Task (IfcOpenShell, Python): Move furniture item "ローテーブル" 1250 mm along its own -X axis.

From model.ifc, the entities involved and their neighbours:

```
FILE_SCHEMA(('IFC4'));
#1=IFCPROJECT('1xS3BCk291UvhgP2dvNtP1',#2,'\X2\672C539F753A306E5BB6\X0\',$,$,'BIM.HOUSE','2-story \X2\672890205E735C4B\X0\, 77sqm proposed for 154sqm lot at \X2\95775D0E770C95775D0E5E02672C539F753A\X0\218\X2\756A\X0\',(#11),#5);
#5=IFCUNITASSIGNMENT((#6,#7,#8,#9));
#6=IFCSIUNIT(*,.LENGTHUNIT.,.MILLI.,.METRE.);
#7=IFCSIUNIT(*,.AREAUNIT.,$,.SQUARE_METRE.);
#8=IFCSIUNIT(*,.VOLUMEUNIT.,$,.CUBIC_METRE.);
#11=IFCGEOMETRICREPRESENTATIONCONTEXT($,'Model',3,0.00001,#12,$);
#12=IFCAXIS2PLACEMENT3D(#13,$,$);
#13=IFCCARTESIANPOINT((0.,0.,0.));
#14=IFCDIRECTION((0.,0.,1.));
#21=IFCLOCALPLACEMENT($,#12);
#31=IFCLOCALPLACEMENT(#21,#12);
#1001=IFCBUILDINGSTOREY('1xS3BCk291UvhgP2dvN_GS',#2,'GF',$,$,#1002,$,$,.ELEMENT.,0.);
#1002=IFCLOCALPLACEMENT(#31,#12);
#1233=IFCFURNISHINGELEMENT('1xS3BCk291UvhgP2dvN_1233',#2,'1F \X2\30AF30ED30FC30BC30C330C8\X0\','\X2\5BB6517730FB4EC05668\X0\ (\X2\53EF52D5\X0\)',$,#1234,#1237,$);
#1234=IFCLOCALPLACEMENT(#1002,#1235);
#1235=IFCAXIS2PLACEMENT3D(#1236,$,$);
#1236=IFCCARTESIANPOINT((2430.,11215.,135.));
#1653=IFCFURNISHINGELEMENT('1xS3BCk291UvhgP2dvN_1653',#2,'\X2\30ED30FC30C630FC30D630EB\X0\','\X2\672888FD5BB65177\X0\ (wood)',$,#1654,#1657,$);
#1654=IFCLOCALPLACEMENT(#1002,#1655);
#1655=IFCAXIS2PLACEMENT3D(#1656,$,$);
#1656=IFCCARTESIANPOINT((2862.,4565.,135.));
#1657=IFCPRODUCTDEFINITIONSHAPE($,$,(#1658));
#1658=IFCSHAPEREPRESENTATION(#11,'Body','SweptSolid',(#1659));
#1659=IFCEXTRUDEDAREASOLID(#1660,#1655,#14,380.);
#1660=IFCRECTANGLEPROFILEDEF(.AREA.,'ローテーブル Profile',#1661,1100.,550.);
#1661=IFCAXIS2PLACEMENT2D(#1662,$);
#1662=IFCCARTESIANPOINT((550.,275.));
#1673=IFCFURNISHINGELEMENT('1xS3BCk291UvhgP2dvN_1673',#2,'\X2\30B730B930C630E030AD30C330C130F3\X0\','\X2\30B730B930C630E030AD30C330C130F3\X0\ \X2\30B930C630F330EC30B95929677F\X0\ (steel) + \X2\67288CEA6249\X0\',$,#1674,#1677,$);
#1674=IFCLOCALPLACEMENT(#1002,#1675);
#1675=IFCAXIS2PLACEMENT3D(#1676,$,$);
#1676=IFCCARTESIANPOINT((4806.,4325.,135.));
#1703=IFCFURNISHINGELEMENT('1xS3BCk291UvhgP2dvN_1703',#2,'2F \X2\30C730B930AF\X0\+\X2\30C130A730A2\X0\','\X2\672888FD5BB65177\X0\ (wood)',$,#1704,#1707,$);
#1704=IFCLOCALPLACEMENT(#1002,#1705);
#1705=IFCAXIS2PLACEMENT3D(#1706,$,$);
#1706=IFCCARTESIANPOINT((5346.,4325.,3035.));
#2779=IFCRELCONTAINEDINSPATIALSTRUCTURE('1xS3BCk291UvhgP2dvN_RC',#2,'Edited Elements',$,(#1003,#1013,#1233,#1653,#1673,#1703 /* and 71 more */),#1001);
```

```python
import ifcopenshell
import ifcopenshell.api.geometry
import ifcopenshell.util.placement
import ifcopenshell.util.unit

model = ifcopenshell.open("model.ifc")
unit_scale = ifcopenshell.util.unit.calculate_unit_scale(model)

item = model.by_guid("1xS3BCk291UvhgP2dvN_1653")
matrix = ifcopenshell.util.placement.get_local_placement(item.ObjectPlacement)
matrix[:3, 3] -= matrix[:3, 0] * 1.25 / unit_scale
ifcopenshell.api.geometry.edit_object_placement(model, product=item, matrix=matrix, is_si=False)

print(ifcopenshell.util.placement.get_local_placement(item.ObjectPlacement).round(3) + 0.0)

model.write("model_rev.ifc")
```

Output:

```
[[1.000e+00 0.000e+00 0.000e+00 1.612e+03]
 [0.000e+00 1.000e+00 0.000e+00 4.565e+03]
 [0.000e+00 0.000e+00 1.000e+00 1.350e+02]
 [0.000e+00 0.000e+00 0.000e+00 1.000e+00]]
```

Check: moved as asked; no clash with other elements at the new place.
